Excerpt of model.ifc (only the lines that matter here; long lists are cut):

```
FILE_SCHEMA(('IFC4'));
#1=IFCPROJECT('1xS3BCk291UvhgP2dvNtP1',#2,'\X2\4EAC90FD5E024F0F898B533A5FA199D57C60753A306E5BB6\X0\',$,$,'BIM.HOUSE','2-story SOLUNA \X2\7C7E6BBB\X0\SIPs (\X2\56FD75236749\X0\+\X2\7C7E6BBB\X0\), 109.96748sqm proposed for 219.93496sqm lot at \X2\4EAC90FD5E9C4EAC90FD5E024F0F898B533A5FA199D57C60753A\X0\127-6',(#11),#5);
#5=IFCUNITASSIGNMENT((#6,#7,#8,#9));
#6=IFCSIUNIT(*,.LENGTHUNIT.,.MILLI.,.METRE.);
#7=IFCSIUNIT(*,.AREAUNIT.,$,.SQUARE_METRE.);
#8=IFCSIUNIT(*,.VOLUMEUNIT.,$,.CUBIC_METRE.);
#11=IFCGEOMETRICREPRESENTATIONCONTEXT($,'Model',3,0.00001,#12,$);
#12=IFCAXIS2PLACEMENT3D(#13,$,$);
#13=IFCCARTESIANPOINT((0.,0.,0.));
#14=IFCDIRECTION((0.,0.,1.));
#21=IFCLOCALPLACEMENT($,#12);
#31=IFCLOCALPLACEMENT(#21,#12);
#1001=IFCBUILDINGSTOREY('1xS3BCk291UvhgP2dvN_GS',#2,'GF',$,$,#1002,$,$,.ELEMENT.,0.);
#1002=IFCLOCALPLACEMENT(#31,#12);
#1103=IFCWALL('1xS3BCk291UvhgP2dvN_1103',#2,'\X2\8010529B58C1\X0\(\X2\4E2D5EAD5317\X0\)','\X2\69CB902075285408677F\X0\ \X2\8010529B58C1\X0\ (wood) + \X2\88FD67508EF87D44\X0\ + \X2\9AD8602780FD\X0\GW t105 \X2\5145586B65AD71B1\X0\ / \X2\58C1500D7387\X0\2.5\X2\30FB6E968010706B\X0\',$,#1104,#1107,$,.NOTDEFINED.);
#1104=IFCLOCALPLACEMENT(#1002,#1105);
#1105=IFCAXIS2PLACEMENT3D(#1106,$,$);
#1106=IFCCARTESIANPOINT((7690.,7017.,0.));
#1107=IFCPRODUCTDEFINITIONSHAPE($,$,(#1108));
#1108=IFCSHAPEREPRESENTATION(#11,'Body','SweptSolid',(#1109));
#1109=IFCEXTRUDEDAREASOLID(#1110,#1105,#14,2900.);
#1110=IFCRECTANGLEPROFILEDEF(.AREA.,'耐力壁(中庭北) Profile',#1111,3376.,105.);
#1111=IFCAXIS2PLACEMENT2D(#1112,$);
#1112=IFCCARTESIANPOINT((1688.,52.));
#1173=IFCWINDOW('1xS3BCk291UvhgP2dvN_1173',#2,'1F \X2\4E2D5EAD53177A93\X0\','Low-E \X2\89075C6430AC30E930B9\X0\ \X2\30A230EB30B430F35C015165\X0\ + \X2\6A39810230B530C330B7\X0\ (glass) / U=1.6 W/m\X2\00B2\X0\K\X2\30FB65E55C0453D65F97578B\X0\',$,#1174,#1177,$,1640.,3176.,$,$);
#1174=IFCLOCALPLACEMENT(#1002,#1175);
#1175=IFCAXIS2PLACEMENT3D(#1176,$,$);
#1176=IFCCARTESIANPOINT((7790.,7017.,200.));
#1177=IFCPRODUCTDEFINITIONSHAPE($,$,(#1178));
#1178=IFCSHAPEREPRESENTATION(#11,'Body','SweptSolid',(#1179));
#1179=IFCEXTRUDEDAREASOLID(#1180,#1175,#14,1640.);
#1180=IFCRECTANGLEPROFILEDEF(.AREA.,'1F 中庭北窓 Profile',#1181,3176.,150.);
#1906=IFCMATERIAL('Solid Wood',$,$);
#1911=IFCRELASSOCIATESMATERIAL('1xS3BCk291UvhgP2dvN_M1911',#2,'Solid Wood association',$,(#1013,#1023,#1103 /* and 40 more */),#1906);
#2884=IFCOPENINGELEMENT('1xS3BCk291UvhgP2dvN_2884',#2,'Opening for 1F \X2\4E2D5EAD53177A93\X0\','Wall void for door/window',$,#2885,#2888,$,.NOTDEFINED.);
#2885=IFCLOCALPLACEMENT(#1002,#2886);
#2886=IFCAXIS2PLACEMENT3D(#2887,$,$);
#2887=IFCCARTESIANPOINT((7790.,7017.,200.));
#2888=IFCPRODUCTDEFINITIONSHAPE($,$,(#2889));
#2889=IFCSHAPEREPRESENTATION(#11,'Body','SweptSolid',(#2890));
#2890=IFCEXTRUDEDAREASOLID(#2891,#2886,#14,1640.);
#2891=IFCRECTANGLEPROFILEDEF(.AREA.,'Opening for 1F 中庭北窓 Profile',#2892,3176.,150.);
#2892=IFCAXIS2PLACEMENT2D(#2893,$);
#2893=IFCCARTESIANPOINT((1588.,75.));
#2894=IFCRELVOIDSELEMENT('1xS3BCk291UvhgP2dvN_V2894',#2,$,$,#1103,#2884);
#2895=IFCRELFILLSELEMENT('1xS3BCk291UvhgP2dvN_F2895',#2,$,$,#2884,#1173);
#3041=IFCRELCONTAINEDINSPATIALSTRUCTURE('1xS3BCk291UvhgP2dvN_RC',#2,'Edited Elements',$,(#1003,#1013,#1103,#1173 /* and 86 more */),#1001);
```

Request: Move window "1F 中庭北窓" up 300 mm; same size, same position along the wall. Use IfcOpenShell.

```python
import numpy as np
import ifcopenshell
import ifcopenshell.api.geometry
import ifcopenshell.util.placement
import ifcopenshell.util.unit

model = ifcopenshell.open("model.ifc")
unit_scale = ifcopenshell.util.unit.calculate_unit_scale(model)

window = model.by_id(1173)
opening = window.FillsVoids[0].RelatingOpeningElement
dz = 300.0

shift = np.array([0.0, 0.0, dz])
# The window is not placed relative to its opening, so move both.
for product in (opening, window):
    matrix = ifcopenshell.util.placement.get_local_placement(product.ObjectPlacement)
    matrix[:3, 3] += shift
    ifcopenshell.api.geometry.edit_object_placement(model, product=product, matrix=matrix, is_si=False)

print(f"moved by {dz * unit_scale:+.3f} m")

model.write("model-out.ifc")
```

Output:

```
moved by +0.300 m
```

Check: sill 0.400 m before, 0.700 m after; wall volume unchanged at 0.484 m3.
